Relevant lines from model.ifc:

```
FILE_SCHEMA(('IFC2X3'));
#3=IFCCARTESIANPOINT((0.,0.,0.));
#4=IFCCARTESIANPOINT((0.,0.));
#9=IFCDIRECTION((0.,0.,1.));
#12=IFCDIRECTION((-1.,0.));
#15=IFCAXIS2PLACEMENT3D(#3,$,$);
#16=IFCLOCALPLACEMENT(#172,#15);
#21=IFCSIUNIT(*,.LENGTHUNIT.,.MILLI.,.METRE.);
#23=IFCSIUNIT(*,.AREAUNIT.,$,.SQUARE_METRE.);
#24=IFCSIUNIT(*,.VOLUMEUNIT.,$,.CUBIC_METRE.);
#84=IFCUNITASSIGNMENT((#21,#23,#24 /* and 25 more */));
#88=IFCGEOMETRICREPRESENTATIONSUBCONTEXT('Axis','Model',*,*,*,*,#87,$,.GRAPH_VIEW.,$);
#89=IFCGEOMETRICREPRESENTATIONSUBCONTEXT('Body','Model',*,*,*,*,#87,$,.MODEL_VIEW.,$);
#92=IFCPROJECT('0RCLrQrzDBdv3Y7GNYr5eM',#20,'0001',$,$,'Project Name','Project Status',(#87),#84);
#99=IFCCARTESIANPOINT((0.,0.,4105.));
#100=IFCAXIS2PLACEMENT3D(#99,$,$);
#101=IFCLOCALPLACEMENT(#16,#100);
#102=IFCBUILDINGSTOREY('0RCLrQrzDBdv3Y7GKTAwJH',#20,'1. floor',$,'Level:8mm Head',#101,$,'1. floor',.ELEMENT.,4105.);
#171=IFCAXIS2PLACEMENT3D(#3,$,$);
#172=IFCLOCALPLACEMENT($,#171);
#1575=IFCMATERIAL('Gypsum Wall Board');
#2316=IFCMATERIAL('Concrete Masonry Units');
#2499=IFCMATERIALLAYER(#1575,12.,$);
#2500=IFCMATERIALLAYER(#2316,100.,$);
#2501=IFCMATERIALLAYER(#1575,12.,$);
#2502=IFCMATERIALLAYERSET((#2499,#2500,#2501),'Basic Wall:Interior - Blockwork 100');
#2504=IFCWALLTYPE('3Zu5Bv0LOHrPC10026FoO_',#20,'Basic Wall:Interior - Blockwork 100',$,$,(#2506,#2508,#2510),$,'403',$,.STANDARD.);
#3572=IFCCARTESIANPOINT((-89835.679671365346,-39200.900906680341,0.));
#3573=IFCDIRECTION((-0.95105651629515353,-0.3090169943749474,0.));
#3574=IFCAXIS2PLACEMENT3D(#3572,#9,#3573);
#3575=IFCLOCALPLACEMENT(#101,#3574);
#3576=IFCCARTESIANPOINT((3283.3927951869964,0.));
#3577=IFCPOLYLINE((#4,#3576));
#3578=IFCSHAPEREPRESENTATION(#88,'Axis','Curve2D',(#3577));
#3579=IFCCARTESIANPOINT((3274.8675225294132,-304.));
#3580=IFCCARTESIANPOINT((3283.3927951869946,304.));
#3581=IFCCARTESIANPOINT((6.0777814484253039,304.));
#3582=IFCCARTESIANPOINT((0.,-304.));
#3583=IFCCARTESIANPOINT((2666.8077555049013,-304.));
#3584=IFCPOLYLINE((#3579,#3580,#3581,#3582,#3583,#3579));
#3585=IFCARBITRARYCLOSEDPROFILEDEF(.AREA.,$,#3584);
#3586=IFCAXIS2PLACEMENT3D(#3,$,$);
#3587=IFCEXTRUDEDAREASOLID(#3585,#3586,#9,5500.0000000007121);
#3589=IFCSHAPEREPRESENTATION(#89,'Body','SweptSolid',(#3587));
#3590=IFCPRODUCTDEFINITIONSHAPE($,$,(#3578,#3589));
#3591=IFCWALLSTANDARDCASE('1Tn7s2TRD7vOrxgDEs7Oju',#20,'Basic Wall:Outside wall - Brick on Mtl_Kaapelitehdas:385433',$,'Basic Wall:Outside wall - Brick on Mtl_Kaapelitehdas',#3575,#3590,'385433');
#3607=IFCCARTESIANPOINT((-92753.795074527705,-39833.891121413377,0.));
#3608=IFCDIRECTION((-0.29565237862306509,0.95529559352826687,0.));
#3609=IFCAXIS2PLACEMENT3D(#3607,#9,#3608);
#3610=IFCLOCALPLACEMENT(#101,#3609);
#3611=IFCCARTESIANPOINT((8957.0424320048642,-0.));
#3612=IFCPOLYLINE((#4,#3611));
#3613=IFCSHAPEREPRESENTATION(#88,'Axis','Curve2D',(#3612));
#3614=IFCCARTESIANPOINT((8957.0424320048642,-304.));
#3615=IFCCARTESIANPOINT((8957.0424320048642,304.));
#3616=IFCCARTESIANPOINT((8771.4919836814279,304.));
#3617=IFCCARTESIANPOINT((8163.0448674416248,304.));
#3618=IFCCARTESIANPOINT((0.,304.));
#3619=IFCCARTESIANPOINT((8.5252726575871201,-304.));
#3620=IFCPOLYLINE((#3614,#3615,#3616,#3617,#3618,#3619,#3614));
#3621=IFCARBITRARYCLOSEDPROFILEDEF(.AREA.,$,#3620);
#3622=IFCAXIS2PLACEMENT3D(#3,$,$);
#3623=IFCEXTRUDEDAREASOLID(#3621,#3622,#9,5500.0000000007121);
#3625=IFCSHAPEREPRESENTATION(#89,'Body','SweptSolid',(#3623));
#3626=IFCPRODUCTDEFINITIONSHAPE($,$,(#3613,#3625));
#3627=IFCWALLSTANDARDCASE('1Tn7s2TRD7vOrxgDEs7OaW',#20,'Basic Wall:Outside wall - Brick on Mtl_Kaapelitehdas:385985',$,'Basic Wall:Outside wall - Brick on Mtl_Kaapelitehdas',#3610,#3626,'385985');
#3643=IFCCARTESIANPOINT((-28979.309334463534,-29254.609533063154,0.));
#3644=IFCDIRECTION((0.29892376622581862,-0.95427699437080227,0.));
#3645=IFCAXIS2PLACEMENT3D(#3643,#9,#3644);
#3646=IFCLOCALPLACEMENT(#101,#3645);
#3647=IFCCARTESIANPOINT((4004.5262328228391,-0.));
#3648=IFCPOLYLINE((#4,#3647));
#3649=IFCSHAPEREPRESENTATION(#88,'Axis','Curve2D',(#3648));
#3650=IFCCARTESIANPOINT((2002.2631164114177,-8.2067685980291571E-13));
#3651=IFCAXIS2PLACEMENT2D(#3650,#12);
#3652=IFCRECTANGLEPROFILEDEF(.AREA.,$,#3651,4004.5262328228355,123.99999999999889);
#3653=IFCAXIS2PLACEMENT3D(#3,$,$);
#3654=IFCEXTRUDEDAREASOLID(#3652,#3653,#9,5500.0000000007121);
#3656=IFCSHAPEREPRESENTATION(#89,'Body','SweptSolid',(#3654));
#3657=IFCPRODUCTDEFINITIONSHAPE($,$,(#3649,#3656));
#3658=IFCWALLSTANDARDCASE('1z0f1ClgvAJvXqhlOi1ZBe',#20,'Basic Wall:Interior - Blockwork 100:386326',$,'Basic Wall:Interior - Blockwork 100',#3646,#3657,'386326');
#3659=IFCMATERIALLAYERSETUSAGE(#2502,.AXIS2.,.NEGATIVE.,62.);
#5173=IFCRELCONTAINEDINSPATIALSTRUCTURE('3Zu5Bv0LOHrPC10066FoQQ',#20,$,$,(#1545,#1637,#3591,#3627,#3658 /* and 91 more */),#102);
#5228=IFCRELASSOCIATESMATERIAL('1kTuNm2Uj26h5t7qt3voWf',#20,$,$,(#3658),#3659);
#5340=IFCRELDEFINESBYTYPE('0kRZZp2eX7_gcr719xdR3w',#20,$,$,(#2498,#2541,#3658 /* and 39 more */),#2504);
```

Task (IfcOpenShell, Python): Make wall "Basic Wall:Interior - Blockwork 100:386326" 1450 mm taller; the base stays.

```python
import ifcopenshell
import ifcopenshell.geom
import ifcopenshell.util.representation
import ifcopenshell.util.shape

model = ifcopenshell.open("model.ifc")
settings = ifcopenshell.geom.settings()


def volume(element):
    """Net volume in cubic metres, openings subtracted."""
    shape = ifcopenshell.geom.create_shape(settings, element)
    return ifcopenshell.util.shape.get_volume(shape.geometry)


wall = model.by_id(3658)
before = volume(wall)

body = ifcopenshell.util.representation.get_representation(wall, "Model", "Body")
solid = body.Items[0]
old_height = solid.Depth
solid.Depth += 1450.0
after = volume(wall)

print(f"height {old_height:g} -> {solid.Depth:g}, volume {before:.3f} -> {after:.3f} m3")

model.write("model-out.ifc")
```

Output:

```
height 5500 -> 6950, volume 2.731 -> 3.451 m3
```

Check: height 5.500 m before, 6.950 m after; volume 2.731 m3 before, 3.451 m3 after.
